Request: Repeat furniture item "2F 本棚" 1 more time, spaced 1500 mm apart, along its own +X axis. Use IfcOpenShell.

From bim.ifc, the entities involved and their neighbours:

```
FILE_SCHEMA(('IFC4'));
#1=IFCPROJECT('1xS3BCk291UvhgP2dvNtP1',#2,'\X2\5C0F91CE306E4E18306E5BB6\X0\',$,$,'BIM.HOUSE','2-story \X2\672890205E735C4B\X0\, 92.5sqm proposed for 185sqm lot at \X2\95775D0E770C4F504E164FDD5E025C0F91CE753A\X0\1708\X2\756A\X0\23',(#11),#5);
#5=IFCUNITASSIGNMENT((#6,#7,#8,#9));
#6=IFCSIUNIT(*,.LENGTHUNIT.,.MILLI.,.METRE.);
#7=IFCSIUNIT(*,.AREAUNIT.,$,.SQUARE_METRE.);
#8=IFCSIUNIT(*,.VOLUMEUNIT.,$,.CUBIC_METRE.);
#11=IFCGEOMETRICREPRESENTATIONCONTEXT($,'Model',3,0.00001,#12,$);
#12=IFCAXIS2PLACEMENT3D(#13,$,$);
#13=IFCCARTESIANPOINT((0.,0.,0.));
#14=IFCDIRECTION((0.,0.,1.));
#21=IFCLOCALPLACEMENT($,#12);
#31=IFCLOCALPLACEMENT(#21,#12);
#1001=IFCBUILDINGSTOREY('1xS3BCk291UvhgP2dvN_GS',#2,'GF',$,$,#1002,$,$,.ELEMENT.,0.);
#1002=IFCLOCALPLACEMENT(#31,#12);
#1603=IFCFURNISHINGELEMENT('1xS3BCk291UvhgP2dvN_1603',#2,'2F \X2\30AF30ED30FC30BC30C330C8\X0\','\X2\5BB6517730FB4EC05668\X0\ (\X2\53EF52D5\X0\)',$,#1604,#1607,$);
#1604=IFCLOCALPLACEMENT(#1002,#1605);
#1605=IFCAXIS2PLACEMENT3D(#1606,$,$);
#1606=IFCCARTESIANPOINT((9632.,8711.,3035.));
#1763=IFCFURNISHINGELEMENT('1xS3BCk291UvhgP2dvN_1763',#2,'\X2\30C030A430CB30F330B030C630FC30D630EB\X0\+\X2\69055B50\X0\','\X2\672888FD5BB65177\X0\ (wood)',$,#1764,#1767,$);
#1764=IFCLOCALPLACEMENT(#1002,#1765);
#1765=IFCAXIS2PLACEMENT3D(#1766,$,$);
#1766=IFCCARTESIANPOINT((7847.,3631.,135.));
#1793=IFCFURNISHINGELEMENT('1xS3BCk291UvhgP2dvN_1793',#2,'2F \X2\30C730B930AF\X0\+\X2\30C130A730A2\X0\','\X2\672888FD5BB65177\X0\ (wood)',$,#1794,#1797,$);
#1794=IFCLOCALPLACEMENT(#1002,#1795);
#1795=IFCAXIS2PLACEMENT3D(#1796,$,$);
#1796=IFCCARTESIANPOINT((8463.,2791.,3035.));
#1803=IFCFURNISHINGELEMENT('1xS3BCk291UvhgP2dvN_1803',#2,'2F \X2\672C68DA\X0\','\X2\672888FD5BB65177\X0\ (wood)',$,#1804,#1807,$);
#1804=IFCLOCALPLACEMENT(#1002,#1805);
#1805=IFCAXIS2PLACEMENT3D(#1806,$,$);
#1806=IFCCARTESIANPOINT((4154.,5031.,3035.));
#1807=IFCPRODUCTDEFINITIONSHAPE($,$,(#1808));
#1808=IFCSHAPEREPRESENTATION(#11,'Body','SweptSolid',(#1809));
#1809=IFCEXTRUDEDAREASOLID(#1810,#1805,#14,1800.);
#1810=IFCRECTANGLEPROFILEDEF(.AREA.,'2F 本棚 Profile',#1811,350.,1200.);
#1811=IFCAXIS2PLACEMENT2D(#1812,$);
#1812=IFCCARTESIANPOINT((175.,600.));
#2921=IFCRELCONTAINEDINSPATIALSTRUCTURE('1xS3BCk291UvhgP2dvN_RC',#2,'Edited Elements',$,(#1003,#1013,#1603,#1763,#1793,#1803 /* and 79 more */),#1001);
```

```python
import ifcopenshell
import ifcopenshell.api.geometry
import ifcopenshell.api.root
import ifcopenshell.util.element
import ifcopenshell.util.placement

model = ifcopenshell.open("bim.ifc")


def reuse_history(source, copy):
    """copy_class also copies each property set's owner history, people and application; keep the originals."""
    for rel in copy.IsDefinedBy:
        if rel.is_a("IfcRelDefinesByProperties") and (history := rel.RelatingPropertyDefinition.OwnerHistory):
            rel.RelatingPropertyDefinition.OwnerHistory = source.OwnerHistory
            ifcopenshell.util.element.remove_deep2(model, history)


source = model.by_guid("1xS3BCk291UvhgP2dvN_1803")
base = ifcopenshell.util.placement.get_local_placement(source.ObjectPlacement)
step = base[:3, 0] * 1500.0

for i in range(1, 2):
    copy = ifcopenshell.api.root.copy_class(model, product=source)
    copy.Representation = ifcopenshell.util.element.copy_deep(
        model, source.Representation, exclude=["IfcGeometricRepresentationContext", "IfcRepresentationMap"]
    )
    reuse_history(source, copy)
    matrix = base.copy()
    matrix[:3, 3] += i * step
    print("added at", matrix[:3, 3].round(3) + 0.0)
    ifcopenshell.api.geometry.edit_object_placement(model, product=copy, matrix=matrix, is_si=False)

model.write("bim_edited.ifc")
```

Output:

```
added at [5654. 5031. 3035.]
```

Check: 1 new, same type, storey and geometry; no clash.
